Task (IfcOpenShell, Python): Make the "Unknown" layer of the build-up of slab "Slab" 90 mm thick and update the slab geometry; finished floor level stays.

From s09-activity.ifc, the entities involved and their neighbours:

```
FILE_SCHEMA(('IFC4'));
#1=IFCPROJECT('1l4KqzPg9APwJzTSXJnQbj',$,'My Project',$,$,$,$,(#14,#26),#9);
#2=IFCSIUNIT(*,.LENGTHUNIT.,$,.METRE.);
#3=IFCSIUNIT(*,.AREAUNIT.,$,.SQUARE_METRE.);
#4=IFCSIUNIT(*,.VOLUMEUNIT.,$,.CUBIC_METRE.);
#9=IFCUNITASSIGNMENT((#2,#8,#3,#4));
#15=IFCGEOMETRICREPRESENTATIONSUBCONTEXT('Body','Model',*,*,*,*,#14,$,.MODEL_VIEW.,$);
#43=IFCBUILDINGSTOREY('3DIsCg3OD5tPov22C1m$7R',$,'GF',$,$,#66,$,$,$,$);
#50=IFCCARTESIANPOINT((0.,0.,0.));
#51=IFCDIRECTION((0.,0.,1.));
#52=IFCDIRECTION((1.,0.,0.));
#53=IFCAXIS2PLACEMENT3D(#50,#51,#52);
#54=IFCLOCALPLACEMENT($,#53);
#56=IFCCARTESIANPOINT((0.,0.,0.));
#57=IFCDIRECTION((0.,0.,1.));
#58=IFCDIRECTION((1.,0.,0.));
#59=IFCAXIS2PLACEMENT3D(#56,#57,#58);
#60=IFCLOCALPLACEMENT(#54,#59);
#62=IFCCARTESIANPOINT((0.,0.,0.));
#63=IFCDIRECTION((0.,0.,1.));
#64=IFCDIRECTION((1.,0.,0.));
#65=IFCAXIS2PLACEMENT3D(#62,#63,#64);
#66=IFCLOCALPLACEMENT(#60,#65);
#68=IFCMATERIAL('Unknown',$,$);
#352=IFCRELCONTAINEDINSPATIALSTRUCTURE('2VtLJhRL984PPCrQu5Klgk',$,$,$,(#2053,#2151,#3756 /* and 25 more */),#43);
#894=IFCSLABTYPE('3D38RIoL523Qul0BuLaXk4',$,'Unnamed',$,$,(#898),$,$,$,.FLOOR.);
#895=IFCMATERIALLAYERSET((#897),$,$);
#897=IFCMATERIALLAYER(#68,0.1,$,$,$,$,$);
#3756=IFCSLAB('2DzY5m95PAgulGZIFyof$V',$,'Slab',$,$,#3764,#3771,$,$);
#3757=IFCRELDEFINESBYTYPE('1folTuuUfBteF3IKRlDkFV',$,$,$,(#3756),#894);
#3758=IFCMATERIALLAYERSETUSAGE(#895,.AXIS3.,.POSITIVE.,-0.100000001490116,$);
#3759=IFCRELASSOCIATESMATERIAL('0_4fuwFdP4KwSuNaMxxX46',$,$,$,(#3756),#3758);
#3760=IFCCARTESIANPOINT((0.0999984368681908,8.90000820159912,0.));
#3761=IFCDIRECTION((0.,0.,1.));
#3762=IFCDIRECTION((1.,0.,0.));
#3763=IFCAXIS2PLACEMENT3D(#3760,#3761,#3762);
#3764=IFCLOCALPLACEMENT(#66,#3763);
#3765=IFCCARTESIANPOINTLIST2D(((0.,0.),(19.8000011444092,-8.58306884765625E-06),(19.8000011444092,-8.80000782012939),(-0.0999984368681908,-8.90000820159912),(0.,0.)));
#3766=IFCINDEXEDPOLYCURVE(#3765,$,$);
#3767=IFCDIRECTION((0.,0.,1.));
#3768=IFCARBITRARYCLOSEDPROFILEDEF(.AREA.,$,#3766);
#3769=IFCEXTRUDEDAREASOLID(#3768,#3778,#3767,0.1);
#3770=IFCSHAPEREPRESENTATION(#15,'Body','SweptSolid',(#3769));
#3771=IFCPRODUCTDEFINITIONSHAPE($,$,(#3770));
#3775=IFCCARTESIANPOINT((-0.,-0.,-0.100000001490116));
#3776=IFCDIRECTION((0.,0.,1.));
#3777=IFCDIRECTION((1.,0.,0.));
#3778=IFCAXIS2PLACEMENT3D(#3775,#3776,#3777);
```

```python
import ifcopenshell
import ifcopenshell.util.element
import ifcopenshell.util.representation
import ifcopenshell.util.unit

model = ifcopenshell.open("s09-activity.ifc")
unit_scale = ifcopenshell.util.unit.calculate_unit_scale(model)

layer_set = model.by_id(895)
layer = next(l for l in layer_set.MaterialLayers if l.Material and l.Material.Name == "Unknown")
change = 0.09 / unit_scale - layer.LayerThickness
layer.LayerThickness += change

# Geometry does not follow the layer set by itself.
slabs = [e for e in ifcopenshell.util.element.get_elements_by_material(model, layer_set) if e.is_a("IfcSlab")]
for slab in sorted(slabs, key=lambda e: e.id()):
    body = ifcopenshell.util.representation.get_representation(slab, "Model", "Body")
    solid = body.Items[0]
    old_depth = solid.Depth
    solid.Depth += change
    # Extruded upwards: lower the start of the extrusion so the top stays.
    x, y, z = solid.Position.Location.Coordinates
    solid.Position.Location = model.createIfcCartesianPoint((x, y, z - change))
    print(slab.id(), f"{old_depth:g} -> {solid.Depth:g}")

# The layers are counted up from the underside, which has moved.
for usage in {ifcopenshell.util.element.get_material(slab) for slab in slabs}:
    usage.OffsetFromReferenceLine -= change

model.write("s09-activity_rev.ifc")
```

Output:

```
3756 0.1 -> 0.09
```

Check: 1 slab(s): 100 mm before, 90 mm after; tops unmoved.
